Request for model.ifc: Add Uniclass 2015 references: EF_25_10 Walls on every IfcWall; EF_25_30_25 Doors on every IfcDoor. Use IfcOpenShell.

First a look at what the model holds.

```python
import ifcopenshell

model = ifcopenshell.open("model.ifc")
print(model.schema)
print("classifications:", [c.Name for c in model.by_type("IfcClassification")])
for ifc_class in ("IfcDoor", "IfcRoof", "IfcStair", "IfcWall", "IfcWindow"):
    print(ifc_class, len(model.by_type(ifc_class)))
```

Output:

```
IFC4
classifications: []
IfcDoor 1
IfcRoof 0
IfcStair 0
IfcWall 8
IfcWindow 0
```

```python
import ifcopenshell
import ifcopenshell.api.classification

model = ifcopenshell.open("model.ifc")

system = ifcopenshell.api.classification.add_classification(model, classification="Uniclass 2015")

codes = {
    "IfcWall": ("EF_25_10", "Walls"),
    "IfcDoor": ("EF_25_30_25", "Doors"),
}
for ifc_class, (code, name) in codes.items():
    products = model.by_type(ifc_class)
    ifcopenshell.api.classification.add_reference(
        model, products=products, classification=system, identification=code, name=name
    )
    print(code, len(products))

model.write("model_edited.ifc")
```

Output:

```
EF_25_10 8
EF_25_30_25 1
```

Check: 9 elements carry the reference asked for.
